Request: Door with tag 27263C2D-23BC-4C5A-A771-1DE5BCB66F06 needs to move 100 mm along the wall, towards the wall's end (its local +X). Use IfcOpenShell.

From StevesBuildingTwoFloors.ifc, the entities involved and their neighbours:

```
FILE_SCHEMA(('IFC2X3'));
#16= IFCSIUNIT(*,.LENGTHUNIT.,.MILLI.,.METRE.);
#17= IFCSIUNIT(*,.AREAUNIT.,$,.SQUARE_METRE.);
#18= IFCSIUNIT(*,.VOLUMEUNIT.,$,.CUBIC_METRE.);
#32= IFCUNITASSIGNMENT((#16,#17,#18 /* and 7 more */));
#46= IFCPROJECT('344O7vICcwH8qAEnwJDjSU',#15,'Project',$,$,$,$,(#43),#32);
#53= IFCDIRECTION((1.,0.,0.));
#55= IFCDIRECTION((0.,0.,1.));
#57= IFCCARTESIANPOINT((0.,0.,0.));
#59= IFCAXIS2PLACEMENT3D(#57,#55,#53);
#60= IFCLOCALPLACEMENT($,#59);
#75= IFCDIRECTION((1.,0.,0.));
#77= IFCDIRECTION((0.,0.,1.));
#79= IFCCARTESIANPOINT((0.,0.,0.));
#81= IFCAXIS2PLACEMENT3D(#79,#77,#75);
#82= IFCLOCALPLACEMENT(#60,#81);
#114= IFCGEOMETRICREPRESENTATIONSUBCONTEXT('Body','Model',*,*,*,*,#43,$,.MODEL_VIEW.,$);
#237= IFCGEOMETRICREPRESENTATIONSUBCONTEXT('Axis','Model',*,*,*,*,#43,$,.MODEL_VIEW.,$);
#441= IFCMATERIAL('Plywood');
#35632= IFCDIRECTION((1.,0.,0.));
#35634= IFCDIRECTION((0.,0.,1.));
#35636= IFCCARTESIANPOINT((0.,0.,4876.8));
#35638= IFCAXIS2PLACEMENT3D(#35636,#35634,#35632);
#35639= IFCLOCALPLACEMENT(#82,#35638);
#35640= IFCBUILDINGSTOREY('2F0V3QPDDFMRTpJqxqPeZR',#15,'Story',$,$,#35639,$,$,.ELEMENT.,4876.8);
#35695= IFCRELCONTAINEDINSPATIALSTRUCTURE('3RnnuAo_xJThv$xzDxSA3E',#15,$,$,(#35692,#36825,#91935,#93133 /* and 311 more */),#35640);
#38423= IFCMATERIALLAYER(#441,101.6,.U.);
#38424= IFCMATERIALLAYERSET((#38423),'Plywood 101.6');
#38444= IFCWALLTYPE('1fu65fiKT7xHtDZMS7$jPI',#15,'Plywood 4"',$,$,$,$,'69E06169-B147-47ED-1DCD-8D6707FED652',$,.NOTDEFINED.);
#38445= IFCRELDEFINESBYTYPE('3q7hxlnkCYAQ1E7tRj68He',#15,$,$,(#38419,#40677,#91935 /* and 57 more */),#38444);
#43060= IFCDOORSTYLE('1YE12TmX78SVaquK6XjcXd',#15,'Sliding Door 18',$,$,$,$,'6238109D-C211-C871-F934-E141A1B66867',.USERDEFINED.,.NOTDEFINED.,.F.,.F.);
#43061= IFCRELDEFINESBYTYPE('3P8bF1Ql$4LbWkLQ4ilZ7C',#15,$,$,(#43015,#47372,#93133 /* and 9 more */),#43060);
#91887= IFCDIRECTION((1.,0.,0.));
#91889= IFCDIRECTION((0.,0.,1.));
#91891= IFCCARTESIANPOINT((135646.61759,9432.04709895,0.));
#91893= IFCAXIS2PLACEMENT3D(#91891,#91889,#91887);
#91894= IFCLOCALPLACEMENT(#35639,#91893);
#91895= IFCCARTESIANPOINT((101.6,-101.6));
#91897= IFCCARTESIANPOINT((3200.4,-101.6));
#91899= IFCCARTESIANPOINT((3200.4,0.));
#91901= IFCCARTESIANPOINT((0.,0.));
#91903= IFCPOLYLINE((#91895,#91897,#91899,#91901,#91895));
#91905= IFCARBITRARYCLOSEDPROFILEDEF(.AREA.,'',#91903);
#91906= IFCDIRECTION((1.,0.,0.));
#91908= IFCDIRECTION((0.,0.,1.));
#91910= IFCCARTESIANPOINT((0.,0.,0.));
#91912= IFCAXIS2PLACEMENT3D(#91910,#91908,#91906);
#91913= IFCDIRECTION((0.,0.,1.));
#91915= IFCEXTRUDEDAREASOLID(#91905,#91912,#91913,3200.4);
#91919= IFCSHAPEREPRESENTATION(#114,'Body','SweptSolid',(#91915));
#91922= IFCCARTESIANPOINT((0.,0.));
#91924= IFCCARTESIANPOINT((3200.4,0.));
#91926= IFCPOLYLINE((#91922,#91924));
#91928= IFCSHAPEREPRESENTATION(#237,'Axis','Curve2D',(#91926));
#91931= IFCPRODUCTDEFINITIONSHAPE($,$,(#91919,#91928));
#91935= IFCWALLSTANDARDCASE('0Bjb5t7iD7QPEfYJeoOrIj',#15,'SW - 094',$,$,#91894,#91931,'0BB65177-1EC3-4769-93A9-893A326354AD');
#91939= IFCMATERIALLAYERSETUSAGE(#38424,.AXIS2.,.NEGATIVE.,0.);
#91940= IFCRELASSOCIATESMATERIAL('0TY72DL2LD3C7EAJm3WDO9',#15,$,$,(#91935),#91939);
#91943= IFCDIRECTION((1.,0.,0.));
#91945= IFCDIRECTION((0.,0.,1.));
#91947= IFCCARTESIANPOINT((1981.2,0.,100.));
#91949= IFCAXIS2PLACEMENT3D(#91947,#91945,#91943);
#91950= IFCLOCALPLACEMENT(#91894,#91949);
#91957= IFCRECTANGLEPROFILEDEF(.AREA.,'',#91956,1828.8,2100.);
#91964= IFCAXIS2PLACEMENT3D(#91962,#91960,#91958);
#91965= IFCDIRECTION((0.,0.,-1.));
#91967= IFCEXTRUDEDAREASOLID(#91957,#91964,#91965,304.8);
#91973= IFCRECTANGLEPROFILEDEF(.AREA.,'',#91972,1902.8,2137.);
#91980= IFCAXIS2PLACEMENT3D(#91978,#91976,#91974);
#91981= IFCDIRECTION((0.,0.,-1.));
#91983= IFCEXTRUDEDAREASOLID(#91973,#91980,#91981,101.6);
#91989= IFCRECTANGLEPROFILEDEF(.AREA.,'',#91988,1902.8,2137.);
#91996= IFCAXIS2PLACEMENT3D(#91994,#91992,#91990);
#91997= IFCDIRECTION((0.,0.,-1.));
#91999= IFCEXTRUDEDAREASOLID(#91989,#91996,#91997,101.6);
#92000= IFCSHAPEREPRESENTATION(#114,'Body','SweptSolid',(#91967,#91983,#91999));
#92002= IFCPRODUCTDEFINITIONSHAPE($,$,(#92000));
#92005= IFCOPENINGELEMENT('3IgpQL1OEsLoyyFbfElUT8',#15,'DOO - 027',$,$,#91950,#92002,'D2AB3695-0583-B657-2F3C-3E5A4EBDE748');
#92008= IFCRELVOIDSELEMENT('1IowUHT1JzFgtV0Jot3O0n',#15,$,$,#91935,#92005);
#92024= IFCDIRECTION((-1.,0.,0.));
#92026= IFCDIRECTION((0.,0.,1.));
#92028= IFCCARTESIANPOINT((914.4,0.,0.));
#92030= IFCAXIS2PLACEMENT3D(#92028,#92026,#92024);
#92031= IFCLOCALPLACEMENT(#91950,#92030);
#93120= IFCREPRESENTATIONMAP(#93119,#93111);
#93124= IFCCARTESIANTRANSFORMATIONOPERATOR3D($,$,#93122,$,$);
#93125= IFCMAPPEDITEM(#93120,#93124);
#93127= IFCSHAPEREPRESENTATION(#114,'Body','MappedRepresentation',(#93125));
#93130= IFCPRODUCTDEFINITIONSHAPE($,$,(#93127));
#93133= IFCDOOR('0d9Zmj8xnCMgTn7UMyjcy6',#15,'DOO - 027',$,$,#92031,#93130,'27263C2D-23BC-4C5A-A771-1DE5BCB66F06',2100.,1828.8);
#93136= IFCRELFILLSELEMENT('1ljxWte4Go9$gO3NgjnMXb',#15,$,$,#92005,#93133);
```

```python
import ifcopenshell
import ifcopenshell.api.geometry
import ifcopenshell.util.placement

model = ifcopenshell.open("StevesBuildingTwoFloors.ifc")

door = model.by_guid("0d9Zmj8xnCMgTn7UMyjcy6")
opening = door.FillsVoids[0].RelatingOpeningElement
wall = opening.VoidsElements[0].RelatingBuildingElement

wall_matrix = ifcopenshell.util.placement.get_local_placement(wall.ObjectPlacement)
shift = wall_matrix[:3, 0] * 100.0
before = ifcopenshell.util.placement.get_local_placement(door.ObjectPlacement)[:3, 3].copy()

# The door is placed relative to its opening, so it follows when the opening moves.
matrix = ifcopenshell.util.placement.get_local_placement(opening.ObjectPlacement)
matrix[:3, 3] += shift
ifcopenshell.api.geometry.edit_object_placement(
    model, product=opening, matrix=matrix, is_si=False, should_transform_children=True
)

after = ifcopenshell.util.placement.get_local_placement(door.ObjectPlacement)[:3, 3]
print("door moved by", (after - before).round(3) + 0.0)

model.write("StevesBuildingTwoFloors_edited.ifc")
```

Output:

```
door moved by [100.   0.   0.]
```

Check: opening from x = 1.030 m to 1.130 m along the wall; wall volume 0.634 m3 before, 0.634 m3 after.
